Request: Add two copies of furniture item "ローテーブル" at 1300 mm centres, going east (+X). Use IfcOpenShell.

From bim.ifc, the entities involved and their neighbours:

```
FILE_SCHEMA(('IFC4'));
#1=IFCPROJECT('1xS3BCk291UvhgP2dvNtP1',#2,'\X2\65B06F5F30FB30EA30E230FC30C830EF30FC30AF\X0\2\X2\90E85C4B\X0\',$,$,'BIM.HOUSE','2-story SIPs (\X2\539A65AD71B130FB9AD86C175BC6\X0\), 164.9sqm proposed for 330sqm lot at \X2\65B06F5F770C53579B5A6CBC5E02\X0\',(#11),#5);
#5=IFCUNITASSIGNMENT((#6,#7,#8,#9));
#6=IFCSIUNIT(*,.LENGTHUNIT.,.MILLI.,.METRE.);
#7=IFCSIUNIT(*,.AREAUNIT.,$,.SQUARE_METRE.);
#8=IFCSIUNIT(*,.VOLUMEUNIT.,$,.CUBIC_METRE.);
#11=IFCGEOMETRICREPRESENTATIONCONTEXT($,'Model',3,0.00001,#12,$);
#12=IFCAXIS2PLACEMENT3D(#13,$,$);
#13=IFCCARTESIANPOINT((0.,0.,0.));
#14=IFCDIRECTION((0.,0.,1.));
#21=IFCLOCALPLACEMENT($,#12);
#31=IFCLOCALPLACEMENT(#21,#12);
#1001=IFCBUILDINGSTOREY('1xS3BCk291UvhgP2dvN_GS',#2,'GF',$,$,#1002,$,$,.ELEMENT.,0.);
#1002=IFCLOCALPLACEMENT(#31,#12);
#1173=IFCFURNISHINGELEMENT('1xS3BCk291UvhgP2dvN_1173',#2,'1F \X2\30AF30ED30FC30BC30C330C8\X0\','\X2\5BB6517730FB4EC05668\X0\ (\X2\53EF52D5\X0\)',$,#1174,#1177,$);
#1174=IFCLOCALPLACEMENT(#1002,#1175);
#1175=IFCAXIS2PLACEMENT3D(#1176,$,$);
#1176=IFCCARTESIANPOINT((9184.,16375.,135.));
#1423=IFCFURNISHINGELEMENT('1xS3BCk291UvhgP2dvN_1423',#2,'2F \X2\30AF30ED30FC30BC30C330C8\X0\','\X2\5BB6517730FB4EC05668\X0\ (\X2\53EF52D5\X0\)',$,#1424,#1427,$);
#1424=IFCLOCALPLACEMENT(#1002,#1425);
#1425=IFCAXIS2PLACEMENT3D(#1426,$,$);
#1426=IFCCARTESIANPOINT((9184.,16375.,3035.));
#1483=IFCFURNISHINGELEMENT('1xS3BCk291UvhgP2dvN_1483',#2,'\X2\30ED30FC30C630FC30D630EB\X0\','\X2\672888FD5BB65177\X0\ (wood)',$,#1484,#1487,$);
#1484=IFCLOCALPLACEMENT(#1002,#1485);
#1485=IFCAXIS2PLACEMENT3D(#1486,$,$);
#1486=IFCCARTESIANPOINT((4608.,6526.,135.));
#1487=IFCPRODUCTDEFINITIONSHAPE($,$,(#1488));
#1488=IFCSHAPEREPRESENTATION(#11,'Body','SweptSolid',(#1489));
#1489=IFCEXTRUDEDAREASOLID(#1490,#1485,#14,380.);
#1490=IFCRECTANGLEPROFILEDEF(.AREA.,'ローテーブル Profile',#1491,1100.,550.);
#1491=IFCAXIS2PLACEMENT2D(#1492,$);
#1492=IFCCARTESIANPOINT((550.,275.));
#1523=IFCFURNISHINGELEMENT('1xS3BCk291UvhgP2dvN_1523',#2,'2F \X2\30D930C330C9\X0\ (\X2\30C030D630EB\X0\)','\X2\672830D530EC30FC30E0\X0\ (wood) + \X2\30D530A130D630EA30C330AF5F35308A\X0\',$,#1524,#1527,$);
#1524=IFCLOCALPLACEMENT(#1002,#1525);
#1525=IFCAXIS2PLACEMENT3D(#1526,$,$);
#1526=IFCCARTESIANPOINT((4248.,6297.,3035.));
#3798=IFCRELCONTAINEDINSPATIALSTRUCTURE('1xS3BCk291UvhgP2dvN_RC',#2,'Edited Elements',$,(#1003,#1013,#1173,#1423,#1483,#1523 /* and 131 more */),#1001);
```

```python
import numpy as np
import ifcopenshell
import ifcopenshell.api.geometry
import ifcopenshell.api.root
import ifcopenshell.util.element
import ifcopenshell.util.placement

model = ifcopenshell.open("bim.ifc")


def reuse_history(source, copy):
    """copy_class also copies each property set's owner history, people and application; keep the originals."""
    for rel in copy.IsDefinedBy:
        if rel.is_a("IfcRelDefinesByProperties") and (history := rel.RelatingPropertyDefinition.OwnerHistory):
            rel.RelatingPropertyDefinition.OwnerHistory = source.OwnerHistory
            ifcopenshell.util.element.remove_deep2(model, history)


source = model.by_guid("1xS3BCk291UvhgP2dvN_1483")
base = ifcopenshell.util.placement.get_local_placement(source.ObjectPlacement)
step = np.array([1.0, 0.0, 0.0]) * 1300.0

for i in range(1, 3):
    copy = ifcopenshell.api.root.copy_class(model, product=source)
    copy.Representation = ifcopenshell.util.element.copy_deep(
        model, source.Representation, exclude=["IfcGeometricRepresentationContext", "IfcRepresentationMap"]
    )
    reuse_history(source, copy)
    matrix = base.copy()
    matrix[:3, 3] += i * step
    print("added at", matrix[:3, 3].round(3) + 0.0)
    ifcopenshell.api.geometry.edit_object_placement(model, product=copy, matrix=matrix, is_si=False)

model.write("bim_updated.ifc")
```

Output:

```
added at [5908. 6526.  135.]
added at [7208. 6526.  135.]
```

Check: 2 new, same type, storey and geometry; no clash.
